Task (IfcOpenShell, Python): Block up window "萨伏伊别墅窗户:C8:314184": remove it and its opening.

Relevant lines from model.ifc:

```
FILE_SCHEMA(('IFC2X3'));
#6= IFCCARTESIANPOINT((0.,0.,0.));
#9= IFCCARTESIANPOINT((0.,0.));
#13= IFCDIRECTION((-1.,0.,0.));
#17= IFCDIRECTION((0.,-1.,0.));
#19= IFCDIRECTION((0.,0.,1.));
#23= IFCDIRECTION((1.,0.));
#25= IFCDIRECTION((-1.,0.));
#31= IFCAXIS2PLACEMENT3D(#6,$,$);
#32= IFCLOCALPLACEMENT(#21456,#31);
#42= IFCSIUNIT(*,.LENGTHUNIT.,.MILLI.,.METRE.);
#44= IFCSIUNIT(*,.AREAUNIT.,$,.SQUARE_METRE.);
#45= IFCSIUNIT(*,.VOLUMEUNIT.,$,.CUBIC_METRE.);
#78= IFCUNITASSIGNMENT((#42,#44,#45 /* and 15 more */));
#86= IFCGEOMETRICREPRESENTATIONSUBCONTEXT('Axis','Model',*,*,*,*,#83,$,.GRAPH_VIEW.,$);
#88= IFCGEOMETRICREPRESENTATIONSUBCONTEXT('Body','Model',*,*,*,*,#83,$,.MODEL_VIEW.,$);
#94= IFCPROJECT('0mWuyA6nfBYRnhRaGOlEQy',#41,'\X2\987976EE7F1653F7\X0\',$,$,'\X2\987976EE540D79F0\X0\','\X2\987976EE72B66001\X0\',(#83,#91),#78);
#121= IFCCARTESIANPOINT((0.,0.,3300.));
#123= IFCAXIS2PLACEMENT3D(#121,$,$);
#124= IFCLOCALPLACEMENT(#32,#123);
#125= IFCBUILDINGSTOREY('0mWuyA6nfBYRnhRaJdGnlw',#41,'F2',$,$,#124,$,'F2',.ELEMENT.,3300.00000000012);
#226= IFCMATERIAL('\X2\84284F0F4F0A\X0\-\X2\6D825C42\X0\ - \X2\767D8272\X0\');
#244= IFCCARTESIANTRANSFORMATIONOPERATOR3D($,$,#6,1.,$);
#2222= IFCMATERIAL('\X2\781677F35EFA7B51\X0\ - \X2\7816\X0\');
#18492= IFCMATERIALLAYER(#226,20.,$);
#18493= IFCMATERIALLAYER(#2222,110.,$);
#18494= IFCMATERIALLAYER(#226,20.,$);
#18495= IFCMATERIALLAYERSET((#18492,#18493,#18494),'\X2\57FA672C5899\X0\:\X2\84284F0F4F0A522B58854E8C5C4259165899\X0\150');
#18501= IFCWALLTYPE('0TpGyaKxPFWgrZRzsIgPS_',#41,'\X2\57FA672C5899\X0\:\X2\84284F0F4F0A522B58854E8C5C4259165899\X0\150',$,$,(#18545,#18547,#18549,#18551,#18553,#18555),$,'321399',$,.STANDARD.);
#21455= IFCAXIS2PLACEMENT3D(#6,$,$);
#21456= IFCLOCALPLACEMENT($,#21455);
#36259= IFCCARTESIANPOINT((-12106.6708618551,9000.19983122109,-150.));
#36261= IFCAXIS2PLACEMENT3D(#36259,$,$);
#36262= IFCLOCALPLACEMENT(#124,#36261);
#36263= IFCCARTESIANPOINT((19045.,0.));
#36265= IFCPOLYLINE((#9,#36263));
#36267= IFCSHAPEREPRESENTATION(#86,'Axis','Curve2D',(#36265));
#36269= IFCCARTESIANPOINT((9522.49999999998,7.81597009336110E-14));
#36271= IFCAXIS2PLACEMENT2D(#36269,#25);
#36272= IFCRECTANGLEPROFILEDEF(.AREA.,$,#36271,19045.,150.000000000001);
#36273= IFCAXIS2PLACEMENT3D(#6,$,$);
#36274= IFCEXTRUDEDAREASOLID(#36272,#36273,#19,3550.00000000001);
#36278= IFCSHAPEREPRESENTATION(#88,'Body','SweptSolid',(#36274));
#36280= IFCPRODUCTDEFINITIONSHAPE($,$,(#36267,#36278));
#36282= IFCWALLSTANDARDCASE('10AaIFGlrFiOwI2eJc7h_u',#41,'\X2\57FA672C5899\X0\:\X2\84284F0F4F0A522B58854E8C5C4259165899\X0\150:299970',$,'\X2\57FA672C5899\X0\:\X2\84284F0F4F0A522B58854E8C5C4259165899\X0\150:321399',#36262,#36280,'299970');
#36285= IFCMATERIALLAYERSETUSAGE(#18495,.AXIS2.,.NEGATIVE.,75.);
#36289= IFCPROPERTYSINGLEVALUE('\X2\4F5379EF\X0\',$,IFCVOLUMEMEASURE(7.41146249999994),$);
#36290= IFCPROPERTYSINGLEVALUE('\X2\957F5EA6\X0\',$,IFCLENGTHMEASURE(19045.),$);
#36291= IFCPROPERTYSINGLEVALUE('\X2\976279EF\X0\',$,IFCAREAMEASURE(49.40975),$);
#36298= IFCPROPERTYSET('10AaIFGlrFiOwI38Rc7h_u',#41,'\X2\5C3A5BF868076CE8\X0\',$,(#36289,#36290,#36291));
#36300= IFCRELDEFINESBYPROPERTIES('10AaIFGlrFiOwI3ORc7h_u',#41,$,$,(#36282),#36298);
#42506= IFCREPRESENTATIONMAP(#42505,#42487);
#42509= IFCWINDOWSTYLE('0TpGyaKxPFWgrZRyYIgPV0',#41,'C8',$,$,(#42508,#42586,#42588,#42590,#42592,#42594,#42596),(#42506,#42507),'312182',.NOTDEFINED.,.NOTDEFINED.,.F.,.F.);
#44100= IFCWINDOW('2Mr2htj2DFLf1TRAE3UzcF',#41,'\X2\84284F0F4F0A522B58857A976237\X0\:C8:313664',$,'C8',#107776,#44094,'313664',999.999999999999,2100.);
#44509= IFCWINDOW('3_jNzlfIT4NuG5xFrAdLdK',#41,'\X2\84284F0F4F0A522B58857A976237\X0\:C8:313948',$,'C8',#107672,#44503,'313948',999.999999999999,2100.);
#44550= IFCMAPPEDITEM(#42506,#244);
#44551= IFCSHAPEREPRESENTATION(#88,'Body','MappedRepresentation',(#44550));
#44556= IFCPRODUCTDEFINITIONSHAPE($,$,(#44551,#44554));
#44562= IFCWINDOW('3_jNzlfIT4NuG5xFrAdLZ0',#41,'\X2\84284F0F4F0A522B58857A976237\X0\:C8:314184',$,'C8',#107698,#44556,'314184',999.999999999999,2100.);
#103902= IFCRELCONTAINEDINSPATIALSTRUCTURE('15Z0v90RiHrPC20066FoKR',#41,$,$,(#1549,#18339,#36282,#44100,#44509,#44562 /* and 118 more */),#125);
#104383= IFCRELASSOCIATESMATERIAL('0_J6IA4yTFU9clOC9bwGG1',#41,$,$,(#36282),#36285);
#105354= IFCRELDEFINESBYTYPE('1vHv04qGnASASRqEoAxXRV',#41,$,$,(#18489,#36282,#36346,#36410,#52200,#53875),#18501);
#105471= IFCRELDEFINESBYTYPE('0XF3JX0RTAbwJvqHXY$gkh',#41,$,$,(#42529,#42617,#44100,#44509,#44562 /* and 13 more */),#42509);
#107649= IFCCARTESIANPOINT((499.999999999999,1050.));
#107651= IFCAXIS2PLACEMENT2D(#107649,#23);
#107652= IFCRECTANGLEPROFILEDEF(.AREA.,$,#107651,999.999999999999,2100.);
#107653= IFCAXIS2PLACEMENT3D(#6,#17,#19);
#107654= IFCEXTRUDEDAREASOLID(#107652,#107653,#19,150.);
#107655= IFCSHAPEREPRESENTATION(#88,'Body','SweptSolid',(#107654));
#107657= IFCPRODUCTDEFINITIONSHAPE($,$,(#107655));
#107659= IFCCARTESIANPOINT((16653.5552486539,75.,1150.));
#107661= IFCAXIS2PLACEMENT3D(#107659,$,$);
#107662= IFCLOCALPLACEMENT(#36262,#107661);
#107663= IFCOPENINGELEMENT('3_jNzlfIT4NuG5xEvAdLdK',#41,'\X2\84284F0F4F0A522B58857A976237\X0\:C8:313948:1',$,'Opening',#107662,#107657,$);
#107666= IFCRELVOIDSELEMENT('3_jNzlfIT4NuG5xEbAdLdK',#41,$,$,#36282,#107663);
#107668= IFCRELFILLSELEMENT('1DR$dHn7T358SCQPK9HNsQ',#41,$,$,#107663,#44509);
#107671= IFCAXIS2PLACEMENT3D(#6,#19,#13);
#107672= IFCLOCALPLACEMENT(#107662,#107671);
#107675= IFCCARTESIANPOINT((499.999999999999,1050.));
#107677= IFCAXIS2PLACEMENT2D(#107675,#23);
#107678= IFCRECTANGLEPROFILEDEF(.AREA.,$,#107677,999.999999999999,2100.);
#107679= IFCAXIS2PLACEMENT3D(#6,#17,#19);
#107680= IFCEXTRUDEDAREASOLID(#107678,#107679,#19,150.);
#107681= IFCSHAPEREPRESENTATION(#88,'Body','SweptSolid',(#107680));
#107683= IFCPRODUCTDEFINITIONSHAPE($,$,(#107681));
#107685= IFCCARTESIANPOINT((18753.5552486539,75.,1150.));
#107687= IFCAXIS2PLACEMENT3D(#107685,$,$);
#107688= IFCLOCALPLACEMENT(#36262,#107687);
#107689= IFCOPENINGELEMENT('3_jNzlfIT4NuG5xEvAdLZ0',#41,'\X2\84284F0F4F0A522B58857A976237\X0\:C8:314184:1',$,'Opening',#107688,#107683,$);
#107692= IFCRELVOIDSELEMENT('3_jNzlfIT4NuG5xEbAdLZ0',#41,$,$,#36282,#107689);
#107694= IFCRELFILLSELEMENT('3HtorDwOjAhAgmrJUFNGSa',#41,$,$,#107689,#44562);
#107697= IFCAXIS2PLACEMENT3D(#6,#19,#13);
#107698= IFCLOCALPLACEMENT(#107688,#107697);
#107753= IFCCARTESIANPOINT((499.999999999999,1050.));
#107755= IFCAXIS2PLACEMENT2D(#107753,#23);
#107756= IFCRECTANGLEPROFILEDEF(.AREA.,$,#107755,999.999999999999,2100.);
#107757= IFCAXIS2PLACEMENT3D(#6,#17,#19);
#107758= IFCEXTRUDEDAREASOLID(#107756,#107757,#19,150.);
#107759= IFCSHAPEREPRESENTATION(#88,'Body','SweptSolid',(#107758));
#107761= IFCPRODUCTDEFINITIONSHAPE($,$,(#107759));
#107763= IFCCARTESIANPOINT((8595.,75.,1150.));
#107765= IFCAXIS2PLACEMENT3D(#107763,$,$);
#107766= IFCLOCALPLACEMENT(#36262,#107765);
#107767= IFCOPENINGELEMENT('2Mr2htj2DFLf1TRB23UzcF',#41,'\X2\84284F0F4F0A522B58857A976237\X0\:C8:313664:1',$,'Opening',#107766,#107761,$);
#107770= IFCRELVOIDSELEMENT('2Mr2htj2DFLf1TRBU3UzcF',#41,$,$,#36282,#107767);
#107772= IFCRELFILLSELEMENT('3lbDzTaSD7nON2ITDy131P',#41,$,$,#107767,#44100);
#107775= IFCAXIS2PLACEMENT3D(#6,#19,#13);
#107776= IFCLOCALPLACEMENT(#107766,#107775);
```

```python
import ifcopenshell
import ifcopenshell.api.feature
import ifcopenshell.api.pset
import ifcopenshell.api.root
import ifcopenshell.geom
import ifcopenshell.util.element
import ifcopenshell.util.shape
import ifcopenshell.util.unit

model = ifcopenshell.open("model.ifc")
area_scale = ifcopenshell.util.unit.calculate_unit_scale(model, "AREAUNIT")
volume_scale = ifcopenshell.util.unit.calculate_unit_scale(model, "VOLUMEUNIT")
settings = ifcopenshell.geom.settings()


def volume(element):
    """Net volume in cubic metres, openings subtracted."""
    shape = ifcopenshell.geom.create_shape(settings, element)
    return ifcopenshell.util.shape.get_volume(shape.geometry)


window = model.by_guid("3_jNzlfIT4NuG5xFrAdLZ0")
opening = window.FillsVoids[0].RelatingOpeningElement
wall = opening.VoidsElements[0].RelatingBuildingElement
before = volume(wall)

ifcopenshell.api.root.remove_product(model, product=window)
ifcopenshell.api.feature.remove_feature(model, feature=opening)

after = volume(wall)
thickness = 0.15  # wall thickness in metres

# Update the wall's stored quantities.
pset = model.by_id(ifcopenshell.util.element.get_pset(wall, "尺寸标注", should_inherit=False)["id"])
ifcopenshell.api.pset.edit_pset(model, pset=pset, properties={
    "体积": model.create_entity("IfcVolumeMeasure", after / volume_scale),
    "面积": model.create_entity("IfcAreaMeasure", after / thickness / area_scale),
})

print(f"wall volume {before:.3f} -> {after:.3f} m3")

model.write("model-out.ifc")
```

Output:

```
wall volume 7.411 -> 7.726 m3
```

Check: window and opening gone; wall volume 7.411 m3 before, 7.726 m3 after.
